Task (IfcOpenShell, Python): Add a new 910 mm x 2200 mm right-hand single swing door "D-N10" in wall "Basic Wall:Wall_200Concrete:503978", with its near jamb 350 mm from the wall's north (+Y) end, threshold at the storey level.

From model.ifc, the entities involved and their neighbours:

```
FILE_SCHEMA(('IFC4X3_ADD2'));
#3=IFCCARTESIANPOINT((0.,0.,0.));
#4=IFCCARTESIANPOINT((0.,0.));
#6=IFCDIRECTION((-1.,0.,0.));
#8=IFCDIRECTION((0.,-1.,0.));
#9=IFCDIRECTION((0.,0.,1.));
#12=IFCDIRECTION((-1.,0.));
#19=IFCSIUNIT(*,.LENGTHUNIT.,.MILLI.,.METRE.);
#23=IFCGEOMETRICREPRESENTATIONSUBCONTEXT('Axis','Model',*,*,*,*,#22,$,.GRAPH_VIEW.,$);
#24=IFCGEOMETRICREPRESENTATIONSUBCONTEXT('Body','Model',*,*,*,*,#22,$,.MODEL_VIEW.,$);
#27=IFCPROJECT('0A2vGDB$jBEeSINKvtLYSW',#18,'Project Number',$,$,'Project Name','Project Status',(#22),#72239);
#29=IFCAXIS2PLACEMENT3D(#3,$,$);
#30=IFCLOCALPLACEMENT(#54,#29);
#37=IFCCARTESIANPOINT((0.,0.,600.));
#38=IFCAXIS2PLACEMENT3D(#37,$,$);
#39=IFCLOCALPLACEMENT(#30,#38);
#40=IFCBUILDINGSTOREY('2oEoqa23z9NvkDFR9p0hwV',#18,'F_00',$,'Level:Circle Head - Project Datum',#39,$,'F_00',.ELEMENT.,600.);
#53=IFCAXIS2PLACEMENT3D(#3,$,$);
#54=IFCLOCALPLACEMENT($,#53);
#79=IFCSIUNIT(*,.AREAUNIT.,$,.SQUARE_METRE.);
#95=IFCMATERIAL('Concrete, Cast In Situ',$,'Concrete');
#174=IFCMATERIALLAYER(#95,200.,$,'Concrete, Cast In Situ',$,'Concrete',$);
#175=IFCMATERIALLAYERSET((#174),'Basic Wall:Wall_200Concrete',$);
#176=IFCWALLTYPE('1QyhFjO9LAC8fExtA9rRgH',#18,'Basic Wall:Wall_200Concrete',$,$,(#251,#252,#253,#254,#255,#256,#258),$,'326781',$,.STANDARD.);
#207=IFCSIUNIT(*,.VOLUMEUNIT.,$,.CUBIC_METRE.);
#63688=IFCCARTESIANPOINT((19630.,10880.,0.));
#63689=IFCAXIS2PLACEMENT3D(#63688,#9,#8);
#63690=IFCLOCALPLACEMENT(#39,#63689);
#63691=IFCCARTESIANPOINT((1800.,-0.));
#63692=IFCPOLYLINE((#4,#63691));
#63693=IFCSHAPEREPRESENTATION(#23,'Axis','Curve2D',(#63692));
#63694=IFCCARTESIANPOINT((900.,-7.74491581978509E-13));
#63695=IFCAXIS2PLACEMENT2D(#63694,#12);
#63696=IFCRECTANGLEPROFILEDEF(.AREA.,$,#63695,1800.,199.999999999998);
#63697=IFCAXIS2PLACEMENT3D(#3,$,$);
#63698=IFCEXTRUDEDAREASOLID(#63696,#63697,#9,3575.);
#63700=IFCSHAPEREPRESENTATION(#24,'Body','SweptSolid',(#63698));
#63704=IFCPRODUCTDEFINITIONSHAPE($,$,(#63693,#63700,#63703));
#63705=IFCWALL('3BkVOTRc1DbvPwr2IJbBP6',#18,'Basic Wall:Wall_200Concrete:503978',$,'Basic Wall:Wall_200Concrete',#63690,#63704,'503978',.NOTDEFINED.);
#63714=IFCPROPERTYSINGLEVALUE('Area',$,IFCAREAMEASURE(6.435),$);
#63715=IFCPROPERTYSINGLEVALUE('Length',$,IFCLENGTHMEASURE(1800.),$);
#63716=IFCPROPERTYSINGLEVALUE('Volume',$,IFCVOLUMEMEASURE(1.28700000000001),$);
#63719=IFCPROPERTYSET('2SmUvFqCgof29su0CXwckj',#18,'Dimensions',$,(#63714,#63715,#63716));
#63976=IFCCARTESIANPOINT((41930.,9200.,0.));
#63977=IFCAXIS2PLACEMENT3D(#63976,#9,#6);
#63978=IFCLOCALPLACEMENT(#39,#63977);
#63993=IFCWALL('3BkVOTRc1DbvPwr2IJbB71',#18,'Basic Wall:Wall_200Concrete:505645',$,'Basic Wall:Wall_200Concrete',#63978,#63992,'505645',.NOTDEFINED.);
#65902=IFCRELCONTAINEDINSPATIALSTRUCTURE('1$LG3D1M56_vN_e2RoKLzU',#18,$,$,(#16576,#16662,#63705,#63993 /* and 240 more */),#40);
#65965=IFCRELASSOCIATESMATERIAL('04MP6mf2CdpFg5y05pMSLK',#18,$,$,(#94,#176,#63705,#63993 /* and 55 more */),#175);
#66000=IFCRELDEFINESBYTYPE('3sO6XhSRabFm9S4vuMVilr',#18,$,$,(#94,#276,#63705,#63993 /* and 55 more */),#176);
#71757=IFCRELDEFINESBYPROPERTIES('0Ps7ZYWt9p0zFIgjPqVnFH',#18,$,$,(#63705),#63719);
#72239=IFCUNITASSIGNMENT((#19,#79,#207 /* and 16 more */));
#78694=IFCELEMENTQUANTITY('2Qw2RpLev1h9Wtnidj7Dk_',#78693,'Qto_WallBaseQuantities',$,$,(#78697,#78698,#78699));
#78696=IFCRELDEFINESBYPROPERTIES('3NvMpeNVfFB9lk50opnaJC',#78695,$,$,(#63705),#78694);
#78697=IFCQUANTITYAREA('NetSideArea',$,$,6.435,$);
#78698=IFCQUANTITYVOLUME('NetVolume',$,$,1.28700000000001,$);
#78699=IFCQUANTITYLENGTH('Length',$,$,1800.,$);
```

```python
import numpy as np
import ifcopenshell
import ifcopenshell.api.feature
import ifcopenshell.api.geometry
import ifcopenshell.api.pset
import ifcopenshell.api.root
import ifcopenshell.api.spatial
import ifcopenshell.geom
import ifcopenshell.util.element
import ifcopenshell.util.placement
import ifcopenshell.util.representation
import ifcopenshell.util.shape
import ifcopenshell.util.unit

model = ifcopenshell.open("model.ifc")
unit_scale = ifcopenshell.util.unit.calculate_unit_scale(model)
area_scale = ifcopenshell.util.unit.calculate_unit_scale(model, "AREAUNIT")
volume_scale = ifcopenshell.util.unit.calculate_unit_scale(model, "VOLUMEUNIT")
settings = ifcopenshell.geom.settings()


def volume(element):
    """Net volume in cubic metres, openings subtracted."""
    shape = ifcopenshell.geom.create_shape(settings, element)
    return ifcopenshell.util.shape.get_volume(shape.geometry)


wall = model.by_id(63705)
storey = ifcopenshell.util.element.get_container(wall, ifc_class="IfcBuildingStorey")
context = ifcopenshell.util.representation.get_context(model, "Model", "Body", "MODEL_VIEW")
before = volume(wall)

width, height, from_end, sill = 0.91, 2.2, 0.35, 0.0  # metres

# The wall runs along its own X axis, and the end named is its -X end.
wall_shape = ifcopenshell.geom.create_shape(settings, wall)
x, y, z = ifcopenshell.util.shape.get_vertices(wall_shape.geometry).T
start = x.min() + from_end
face, thickness = float(y.min()), float(y.max() - y.min())
wall_matrix = ifcopenshell.util.placement.get_local_placement(wall.ObjectPlacement)
level = ifcopenshell.util.placement.get_local_placement(storey.ObjectPlacement)[2, 3]


def in_wall(x, y):
    """Placement at x, y metres in the wall's axes, at sill height."""
    matrix = wall_matrix.copy()
    matrix[:, 3] = wall_matrix @ np.array([x / unit_scale, y / unit_scale, 0.0, 1.0])
    matrix[2, 3] = level + sill / unit_scale
    return matrix


# Opening: a box that overshoots both wall faces by 50 mm.
opening = ifcopenshell.api.root.create_entity(model, ifc_class="IfcOpeningElement", predefined_type="OPENING")
box = ifcopenshell.api.geometry.add_wall_representation(
    model, context=context, length=width, height=height, thickness=thickness + 0.1
)
ifcopenshell.api.geometry.assign_representation(model, product=opening, representation=box)
ifcopenshell.api.geometry.edit_object_placement(model, product=opening, matrix=in_wall(start, face - 0.05), is_si=False)
ifcopenshell.api.feature.add_feature(model, feature=opening, element=wall)

door = ifcopenshell.api.root.create_entity(model, ifc_class="IfcDoor", name="D-N10", predefined_type="DOOR")
door.OverallWidth, door.OverallHeight = width / unit_scale, height / unit_scale
door.OperationType = "SINGLE_SWING_RIGHT"
body = ifcopenshell.api.geometry.add_door_representation(
    model,
    context=context,
    overall_width=door.OverallWidth,
    overall_height=door.OverallHeight,
    operation_type="SINGLE_SWING_RIGHT",
    lining_properties={"LiningDepth": thickness / unit_scale, "ThresholdDepth": thickness / unit_scale},
)
ifcopenshell.api.geometry.assign_representation(model, product=door, representation=body)
ifcopenshell.api.spatial.assign_container(model, products=[door], relating_structure=storey)
ifcopenshell.api.feature.add_filling(model, opening=opening, element=door)

# The lining spans the wall, so the door starts at the wall face.
ifcopenshell.api.geometry.edit_object_placement(model, product=door, matrix=in_wall(start, face), is_si=False)

after = volume(wall)

# Update the wall's stored quantities.
pset = model.by_id(ifcopenshell.util.element.get_pset(wall, "Dimensions", should_inherit=False)["id"])
ifcopenshell.api.pset.edit_pset(model, pset=pset, properties={
    "Area": model.create_entity("IfcAreaMeasure", after / thickness / area_scale),
    "Volume": model.create_entity("IfcVolumeMeasure", after / volume_scale),
})
qto = model.by_id(ifcopenshell.util.element.get_pset(wall, "Qto_WallBaseQuantities", should_inherit=False)["id"])
ifcopenshell.api.pset.edit_qto(model, qto=qto, properties={
    "NetSideArea": after / thickness / area_scale,
    "NetVolume": after / volume_scale,
})

print(f"wall volume {before:.3f} -> {after:.3f} m3")

model.write("model_v2.ifc")
```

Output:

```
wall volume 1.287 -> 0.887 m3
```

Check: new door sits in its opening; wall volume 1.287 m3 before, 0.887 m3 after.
